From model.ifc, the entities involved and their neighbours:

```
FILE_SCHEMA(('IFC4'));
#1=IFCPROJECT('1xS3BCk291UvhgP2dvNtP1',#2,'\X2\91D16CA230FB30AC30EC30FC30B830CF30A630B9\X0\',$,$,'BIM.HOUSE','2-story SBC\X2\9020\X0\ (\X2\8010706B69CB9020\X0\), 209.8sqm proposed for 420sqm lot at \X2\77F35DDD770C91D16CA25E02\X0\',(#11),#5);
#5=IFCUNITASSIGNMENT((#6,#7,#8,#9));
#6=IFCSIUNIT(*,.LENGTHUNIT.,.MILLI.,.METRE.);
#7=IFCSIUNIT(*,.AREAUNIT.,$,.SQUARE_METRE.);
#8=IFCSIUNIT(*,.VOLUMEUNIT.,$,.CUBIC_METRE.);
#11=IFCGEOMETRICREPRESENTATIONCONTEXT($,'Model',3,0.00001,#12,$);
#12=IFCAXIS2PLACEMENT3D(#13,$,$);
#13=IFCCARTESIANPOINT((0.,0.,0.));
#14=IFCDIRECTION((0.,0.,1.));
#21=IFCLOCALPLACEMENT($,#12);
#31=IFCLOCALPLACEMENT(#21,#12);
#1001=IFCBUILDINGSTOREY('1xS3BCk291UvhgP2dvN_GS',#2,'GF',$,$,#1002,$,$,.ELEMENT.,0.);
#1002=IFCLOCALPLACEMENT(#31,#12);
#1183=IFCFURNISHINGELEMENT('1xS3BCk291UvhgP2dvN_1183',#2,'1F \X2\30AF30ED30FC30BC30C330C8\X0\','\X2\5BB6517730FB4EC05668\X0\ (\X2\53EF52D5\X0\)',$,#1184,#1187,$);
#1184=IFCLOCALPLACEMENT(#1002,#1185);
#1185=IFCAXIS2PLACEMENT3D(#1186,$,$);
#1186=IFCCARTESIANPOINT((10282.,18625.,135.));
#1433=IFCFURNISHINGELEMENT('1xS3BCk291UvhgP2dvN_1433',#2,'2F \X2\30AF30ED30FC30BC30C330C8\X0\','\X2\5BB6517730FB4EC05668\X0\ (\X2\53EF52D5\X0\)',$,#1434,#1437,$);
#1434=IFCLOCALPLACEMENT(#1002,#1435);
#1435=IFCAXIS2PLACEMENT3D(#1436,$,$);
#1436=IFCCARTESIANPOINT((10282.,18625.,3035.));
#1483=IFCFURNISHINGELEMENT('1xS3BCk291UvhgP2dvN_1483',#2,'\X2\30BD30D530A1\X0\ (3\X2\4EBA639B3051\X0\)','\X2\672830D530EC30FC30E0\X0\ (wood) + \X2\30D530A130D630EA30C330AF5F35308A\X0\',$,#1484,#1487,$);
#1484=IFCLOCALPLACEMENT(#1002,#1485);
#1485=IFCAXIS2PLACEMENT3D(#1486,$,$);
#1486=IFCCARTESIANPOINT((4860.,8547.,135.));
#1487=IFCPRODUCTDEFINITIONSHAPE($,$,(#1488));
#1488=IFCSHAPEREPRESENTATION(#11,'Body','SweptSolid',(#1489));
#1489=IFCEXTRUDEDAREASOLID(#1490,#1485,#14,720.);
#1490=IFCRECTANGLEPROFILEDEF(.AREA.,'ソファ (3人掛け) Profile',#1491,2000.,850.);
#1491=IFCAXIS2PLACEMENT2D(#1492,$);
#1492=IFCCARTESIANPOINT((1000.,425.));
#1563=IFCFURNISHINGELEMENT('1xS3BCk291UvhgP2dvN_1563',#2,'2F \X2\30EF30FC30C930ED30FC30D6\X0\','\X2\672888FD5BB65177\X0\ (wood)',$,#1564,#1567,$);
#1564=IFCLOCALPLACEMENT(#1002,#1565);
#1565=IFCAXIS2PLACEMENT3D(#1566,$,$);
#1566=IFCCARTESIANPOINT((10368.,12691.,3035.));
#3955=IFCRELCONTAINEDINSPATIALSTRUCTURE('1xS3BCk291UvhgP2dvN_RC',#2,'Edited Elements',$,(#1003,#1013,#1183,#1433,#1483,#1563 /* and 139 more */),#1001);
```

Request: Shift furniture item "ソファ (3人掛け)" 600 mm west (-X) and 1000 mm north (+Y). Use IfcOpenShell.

```python
import ifcopenshell
import ifcopenshell.api.geometry
import ifcopenshell.util.placement
import ifcopenshell.util.unit

model = ifcopenshell.open("model.ifc")
unit_scale = ifcopenshell.util.unit.calculate_unit_scale(model)

item = model.by_guid("1xS3BCk291UvhgP2dvN_1483")
matrix = ifcopenshell.util.placement.get_local_placement(item.ObjectPlacement)
matrix[0, 3] -= 0.6 / unit_scale
matrix[1, 3] += 1 / unit_scale
ifcopenshell.api.geometry.edit_object_placement(model, product=item, matrix=matrix, is_si=False)

print(ifcopenshell.util.placement.get_local_placement(item.ObjectPlacement).round(3) + 0.0)

model.write("model_edited.ifc")
```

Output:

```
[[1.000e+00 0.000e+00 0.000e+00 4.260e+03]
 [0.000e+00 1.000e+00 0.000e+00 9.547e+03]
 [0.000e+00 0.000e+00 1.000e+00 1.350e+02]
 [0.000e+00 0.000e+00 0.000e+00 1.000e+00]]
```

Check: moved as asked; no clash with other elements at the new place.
